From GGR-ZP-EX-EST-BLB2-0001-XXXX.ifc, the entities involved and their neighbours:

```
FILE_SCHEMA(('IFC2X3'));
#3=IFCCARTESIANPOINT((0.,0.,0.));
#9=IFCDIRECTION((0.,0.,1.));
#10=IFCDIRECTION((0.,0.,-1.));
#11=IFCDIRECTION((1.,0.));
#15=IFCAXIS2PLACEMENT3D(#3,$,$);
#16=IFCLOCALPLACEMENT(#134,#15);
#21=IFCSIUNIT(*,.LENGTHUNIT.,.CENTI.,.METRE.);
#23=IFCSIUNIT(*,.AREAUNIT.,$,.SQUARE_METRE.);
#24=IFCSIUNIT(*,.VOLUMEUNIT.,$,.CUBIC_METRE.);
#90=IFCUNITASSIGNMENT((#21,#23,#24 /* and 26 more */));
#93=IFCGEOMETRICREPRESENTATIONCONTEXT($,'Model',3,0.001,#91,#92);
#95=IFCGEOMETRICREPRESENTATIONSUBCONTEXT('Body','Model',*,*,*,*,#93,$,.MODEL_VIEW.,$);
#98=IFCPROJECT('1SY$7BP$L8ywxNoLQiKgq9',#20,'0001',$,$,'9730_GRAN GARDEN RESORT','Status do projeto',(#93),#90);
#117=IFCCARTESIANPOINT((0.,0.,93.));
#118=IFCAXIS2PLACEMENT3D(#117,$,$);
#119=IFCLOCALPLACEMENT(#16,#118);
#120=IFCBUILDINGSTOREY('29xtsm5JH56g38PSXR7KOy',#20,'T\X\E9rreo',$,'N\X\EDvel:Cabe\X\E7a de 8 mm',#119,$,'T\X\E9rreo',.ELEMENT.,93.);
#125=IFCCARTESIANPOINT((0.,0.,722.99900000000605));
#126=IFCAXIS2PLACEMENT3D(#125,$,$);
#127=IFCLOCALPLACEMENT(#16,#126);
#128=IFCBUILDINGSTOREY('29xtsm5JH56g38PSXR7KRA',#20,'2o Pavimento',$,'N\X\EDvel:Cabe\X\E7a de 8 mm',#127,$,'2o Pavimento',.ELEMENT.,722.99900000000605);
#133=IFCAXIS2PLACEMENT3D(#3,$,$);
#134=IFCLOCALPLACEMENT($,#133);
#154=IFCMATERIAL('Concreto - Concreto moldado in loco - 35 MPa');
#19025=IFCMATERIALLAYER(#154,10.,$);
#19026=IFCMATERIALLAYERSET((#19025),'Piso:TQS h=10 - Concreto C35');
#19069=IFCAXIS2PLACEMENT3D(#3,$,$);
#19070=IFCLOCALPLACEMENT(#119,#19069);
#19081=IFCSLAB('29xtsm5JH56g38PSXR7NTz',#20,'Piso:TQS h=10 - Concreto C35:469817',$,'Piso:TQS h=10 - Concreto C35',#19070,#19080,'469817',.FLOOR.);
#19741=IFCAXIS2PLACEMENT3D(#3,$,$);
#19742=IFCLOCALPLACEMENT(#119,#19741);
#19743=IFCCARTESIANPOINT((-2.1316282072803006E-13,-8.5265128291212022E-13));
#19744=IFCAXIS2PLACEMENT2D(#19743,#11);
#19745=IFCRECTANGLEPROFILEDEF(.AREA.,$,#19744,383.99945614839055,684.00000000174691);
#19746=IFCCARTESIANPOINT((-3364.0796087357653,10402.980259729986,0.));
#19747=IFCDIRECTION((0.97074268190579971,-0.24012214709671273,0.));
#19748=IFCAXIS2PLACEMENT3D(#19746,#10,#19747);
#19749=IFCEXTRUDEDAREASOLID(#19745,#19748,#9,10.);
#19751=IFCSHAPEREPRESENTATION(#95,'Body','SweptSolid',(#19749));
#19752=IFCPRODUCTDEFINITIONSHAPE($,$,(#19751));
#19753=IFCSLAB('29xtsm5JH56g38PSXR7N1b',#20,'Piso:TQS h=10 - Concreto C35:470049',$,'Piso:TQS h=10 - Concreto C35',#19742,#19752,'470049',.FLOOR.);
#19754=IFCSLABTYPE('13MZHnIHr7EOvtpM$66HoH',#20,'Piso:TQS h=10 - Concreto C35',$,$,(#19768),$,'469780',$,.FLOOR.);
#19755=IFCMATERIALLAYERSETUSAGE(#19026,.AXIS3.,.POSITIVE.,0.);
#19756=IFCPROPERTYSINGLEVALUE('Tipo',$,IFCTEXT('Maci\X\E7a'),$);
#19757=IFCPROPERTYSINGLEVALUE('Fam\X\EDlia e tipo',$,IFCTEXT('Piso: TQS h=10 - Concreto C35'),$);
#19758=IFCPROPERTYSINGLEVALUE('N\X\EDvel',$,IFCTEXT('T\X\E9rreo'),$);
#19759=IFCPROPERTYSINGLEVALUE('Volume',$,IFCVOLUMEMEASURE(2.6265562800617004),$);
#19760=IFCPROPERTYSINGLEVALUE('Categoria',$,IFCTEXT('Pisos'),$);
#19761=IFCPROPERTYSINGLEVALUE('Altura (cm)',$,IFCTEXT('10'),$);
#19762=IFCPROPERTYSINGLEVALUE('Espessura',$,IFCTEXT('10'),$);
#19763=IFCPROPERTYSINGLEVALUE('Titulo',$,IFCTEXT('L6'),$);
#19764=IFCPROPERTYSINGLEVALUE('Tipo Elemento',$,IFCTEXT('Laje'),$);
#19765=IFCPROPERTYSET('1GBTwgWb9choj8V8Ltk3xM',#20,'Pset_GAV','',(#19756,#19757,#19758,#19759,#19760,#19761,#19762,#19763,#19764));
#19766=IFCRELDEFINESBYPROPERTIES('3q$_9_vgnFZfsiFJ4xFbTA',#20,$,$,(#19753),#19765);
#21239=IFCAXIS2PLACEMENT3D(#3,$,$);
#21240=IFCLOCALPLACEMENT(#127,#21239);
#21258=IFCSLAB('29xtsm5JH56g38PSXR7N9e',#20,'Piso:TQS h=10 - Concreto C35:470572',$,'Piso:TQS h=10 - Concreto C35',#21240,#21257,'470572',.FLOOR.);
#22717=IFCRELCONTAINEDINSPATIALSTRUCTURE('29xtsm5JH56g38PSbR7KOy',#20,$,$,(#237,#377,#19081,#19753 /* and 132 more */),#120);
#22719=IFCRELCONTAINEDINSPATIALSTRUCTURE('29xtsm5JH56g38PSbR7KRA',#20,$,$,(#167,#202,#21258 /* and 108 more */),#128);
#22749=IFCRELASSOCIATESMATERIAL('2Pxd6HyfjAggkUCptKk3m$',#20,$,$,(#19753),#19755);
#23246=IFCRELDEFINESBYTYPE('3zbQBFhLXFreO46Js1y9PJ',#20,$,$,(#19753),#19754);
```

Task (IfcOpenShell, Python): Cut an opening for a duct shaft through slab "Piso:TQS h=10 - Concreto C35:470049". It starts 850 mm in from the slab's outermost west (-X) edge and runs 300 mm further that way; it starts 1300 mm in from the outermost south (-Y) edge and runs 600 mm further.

```python
import numpy as np
import ifcopenshell
import ifcopenshell.api.feature
import ifcopenshell.api.geometry
import ifcopenshell.api.pset
import ifcopenshell.api.root
import ifcopenshell.geom
import ifcopenshell.util.element
import ifcopenshell.util.placement
import ifcopenshell.util.representation
import ifcopenshell.util.shape
import ifcopenshell.util.unit

model = ifcopenshell.open("GGR-ZP-EX-EST-BLB2-0001-XXXX.ifc")
unit_scale = ifcopenshell.util.unit.calculate_unit_scale(model)
volume_scale = ifcopenshell.util.unit.calculate_unit_scale(model, "VOLUMEUNIT")
settings = ifcopenshell.geom.settings()


def volume(element):
    """Net volume in cubic metres, openings subtracted."""
    shape = ifcopenshell.geom.create_shape(settings, element)
    return ifcopenshell.util.shape.get_volume(shape.geometry)


slab = model.by_id(19753)
before = volume(slab)

# Extent in the slab's own axes, in metres. The edges named are its -X and -Y sides.
slab_shape = ifcopenshell.geom.create_shape(settings, slab)
vertices = ifcopenshell.util.shape.get_vertices(slab_shape.geometry)
x_min, y_min, bottom = vertices.min(axis=0)
top = vertices[:, 2].max()

opening = ifcopenshell.api.root.create_entity(model, ifc_class="IfcOpeningElement", name="Duct shaft opening")
context = ifcopenshell.util.representation.get_context(model, "Model", "Body", "MODEL_VIEW")
width, depth = 0.3, 0.6
outline = [(0.0, 0.0), (width, 0.0), (width, depth), (0.0, depth), (0.0, 0.0)]
# Overshoot both faces by 50 mm so the cut is clean.
shape = ifcopenshell.api.geometry.add_slab_representation(
    model, context=context, depth=top - bottom + 0.1, polyline=outline
)
ifcopenshell.api.geometry.assign_representation(model, product=opening, representation=shape)

matrix = ifcopenshell.util.placement.get_local_placement(slab.ObjectPlacement)
matrix[:, 3] = matrix @ np.append(np.array([x_min + 0.85, y_min + 1.3, bottom - 0.05]) / unit_scale, 1.0)
ifcopenshell.api.geometry.edit_object_placement(model, product=opening, matrix=matrix, is_si=False)
ifcopenshell.api.feature.add_feature(model, feature=opening, element=slab)

after = volume(slab)

# Update the slab's stored quantities.
pset = model.by_id(ifcopenshell.util.element.get_pset(slab, "Pset_GAV", should_inherit=False)["id"])
ifcopenshell.api.pset.edit_pset(model, pset=pset, properties={
    "Volume": model.create_entity("IfcVolumeMeasure", after / volume_scale),
})

print(f"slab volume {before:.3f} -> {after:.3f} m3")

model.write("GGR-ZP-EX-EST-BLB2-0001-XXXX-out.ifc")
```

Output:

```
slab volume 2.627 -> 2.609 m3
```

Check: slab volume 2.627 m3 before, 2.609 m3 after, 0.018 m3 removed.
